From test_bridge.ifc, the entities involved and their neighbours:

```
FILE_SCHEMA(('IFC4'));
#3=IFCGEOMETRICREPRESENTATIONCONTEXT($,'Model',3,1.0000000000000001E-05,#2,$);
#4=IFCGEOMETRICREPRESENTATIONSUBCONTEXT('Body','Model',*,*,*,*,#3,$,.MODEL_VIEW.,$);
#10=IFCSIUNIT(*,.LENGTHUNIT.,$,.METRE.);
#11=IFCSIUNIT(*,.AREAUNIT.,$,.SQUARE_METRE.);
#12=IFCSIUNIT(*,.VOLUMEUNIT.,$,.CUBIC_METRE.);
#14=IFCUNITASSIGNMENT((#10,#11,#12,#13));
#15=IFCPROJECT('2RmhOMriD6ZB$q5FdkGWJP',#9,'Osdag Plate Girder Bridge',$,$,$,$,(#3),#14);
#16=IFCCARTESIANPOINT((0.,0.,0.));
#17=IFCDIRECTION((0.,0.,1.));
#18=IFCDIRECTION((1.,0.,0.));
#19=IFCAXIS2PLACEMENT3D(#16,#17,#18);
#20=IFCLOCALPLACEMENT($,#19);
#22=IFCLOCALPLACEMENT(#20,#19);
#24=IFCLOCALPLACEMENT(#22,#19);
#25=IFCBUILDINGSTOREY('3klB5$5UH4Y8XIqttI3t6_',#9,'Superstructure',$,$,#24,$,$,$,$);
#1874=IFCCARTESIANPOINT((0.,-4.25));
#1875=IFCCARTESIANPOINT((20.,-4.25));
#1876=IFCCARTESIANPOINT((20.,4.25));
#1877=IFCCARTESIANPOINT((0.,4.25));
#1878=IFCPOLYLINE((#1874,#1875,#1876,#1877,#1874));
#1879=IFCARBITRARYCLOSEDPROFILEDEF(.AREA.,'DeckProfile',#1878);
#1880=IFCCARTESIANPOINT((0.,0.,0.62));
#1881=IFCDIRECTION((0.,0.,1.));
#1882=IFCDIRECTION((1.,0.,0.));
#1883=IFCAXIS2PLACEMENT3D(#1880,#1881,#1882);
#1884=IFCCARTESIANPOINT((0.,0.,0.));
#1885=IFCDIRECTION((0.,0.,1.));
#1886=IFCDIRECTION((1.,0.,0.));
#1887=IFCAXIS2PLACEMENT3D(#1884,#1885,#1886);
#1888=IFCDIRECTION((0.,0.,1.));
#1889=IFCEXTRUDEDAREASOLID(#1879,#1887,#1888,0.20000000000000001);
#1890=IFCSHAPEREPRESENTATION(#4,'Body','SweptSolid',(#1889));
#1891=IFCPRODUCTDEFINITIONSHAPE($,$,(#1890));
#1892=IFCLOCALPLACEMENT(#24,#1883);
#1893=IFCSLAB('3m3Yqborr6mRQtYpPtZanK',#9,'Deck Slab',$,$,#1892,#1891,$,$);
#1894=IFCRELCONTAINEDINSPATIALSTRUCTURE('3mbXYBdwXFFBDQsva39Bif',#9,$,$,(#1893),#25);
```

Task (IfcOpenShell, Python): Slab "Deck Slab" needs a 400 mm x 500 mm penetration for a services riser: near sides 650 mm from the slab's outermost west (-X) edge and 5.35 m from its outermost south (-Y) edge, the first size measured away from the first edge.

```python
import numpy as np
import ifcopenshell
import ifcopenshell.api.feature
import ifcopenshell.api.geometry
import ifcopenshell.api.root
import ifcopenshell.geom
import ifcopenshell.util.placement
import ifcopenshell.util.representation
import ifcopenshell.util.shape
import ifcopenshell.util.unit

model = ifcopenshell.open("test_bridge.ifc")
unit_scale = ifcopenshell.util.unit.calculate_unit_scale(model)
settings = ifcopenshell.geom.settings()


def volume(element):
    """Net volume in cubic metres, openings subtracted."""
    shape = ifcopenshell.geom.create_shape(settings, element)
    return ifcopenshell.util.shape.get_volume(shape.geometry)


slab = model.by_id(1893)
before = volume(slab)

# Extent in the slab's own axes, in metres. The edges named are its -X and -Y sides.
slab_shape = ifcopenshell.geom.create_shape(settings, slab)
vertices = ifcopenshell.util.shape.get_vertices(slab_shape.geometry)
x_min, y_min, bottom = vertices.min(axis=0)
top = vertices[:, 2].max()

opening = ifcopenshell.api.root.create_entity(model, ifc_class="IfcOpeningElement", name="Services riser opening", predefined_type="OPENING")
context = ifcopenshell.util.representation.get_context(model, "Model", "Body", "MODEL_VIEW")
width, depth = 0.4, 0.5
outline = [(0.0, 0.0), (width, 0.0), (width, depth), (0.0, depth), (0.0, 0.0)]
# Overshoot both faces by 50 mm so the cut is clean.
shape = ifcopenshell.api.geometry.add_slab_representation(
    model, context=context, depth=top - bottom + 0.1, polyline=outline
)
ifcopenshell.api.geometry.assign_representation(model, product=opening, representation=shape)

matrix = ifcopenshell.util.placement.get_local_placement(slab.ObjectPlacement)
matrix[:, 3] = matrix @ np.append(np.array([x_min + 0.65, y_min + 5.35, bottom - 0.05]) / unit_scale, 1.0)
ifcopenshell.api.geometry.edit_object_placement(model, product=opening, matrix=matrix, is_si=False)
ifcopenshell.api.feature.add_feature(model, feature=opening, element=slab)

after = volume(slab)

print(f"slab volume {before:.3f} -> {after:.3f} m3")

model.write("test_bridge_rev.ifc")
```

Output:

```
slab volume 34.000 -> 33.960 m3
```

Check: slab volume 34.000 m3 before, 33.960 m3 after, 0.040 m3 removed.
